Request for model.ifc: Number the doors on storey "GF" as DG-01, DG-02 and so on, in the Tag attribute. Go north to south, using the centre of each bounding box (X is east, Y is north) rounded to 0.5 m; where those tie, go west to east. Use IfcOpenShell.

First a look at what the model holds.

```python
import ifcopenshell
import ifcopenshell.util.element
import ifcopenshell.util.placement

model = ifcopenshell.open("model.ifc")
print(model.schema)
storey = next(s for s in model.by_type("IfcBuildingStorey") if s.Name == "GF")
doors = [e for e in ifcopenshell.util.element.get_decomposition(storey) if e.is_a("IfcDoor")]
for e in sorted(doors, key=lambda e: e.id()):
    origin = ifcopenshell.util.placement.get_local_placement(e.ObjectPlacement)[:3, 3]
    print(e.id(), e.Tag, e.Name, origin.round(2) + 0.0, sep=" | ")
```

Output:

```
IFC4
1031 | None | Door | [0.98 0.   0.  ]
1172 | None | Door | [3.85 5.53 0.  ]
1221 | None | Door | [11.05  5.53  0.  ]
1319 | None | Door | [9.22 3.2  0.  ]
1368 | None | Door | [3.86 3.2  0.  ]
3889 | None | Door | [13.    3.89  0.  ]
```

```python
import ifcopenshell
import ifcopenshell.geom
import ifcopenshell.util.element
import ifcopenshell.util.shape

model = ifcopenshell.open("model.ifc")
settings = ifcopenshell.geom.settings()
settings.set("use-world-coords", True)


def centre(element):
    shape = ifcopenshell.geom.create_shape(settings, element)
    return ifcopenshell.util.shape.get_bbox_centroid(shape.geometry)


storey = next(s for s in model.by_type("IfcBuildingStorey") if s.Name == "GF")
doors = [e for e in ifcopenshell.util.element.get_decomposition(storey) if e.is_a("IfcDoor")]

# Insertion points can sit at a corner or the storey origin, so sort by the geometry (in metres).
centres = {e: centre(e) for e in doors}
doors.sort(key=lambda e: (-round(centres[e][1] / 0.5), centres[e][0]))

for i, e in enumerate(doors, start=1):
    number = f"DG-{i:02d}"
    e.Tag = number
    print(e.id(), number)

model.write("model_v2.ifc")
```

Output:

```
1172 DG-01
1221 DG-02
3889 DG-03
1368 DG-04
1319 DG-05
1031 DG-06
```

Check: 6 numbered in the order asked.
